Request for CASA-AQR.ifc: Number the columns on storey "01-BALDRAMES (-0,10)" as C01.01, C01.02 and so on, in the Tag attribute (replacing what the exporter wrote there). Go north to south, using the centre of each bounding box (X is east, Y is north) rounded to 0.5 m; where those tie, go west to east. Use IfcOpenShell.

First a look at what the model holds.

```python
import ifcopenshell
import ifcopenshell.util.element
import ifcopenshell.util.placement

model = ifcopenshell.open("CASA-AQR.ifc")
print(model.schema)
storey = next(s for s in model.by_type("IfcBuildingStorey") if s.Name == "01-BALDRAMES (-0,10)")
columns = [e for e in ifcopenshell.util.element.get_decomposition(storey) if e.is_a("IfcColumn")]
for e in sorted(columns, key=lambda e: e.id()):
    origin = ifcopenshell.util.placement.get_local_placement(e.ObjectPlacement)[:3, 3]
    print(e.id(), e.Tag, e.Name, origin.round(2) + 0.0, sep=" | ")
```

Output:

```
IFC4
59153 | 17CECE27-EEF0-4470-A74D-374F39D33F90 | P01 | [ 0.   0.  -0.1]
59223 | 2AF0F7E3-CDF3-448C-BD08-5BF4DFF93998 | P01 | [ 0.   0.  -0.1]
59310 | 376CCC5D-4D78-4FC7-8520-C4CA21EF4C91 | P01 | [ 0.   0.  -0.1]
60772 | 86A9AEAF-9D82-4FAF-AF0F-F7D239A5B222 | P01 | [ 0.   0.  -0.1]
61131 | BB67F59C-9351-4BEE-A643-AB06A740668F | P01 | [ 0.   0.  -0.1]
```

```python
import ifcopenshell
import ifcopenshell.geom
import ifcopenshell.util.element
import ifcopenshell.util.shape

model = ifcopenshell.open("CASA-AQR.ifc")
settings = ifcopenshell.geom.settings()
settings.set("use-world-coords", True)


def centre(element):
    shape = ifcopenshell.geom.create_shape(settings, element)
    return ifcopenshell.util.shape.get_bbox_centroid(shape.geometry)


storey = next(s for s in model.by_type("IfcBuildingStorey") if s.Name == "01-BALDRAMES (-0,10)")
columns = [e for e in ifcopenshell.util.element.get_decomposition(storey) if e.is_a("IfcColumn")]

# Insertion points can sit at a corner or the storey origin, so sort by the geometry (in metres).
centres = {e: centre(e) for e in columns}
columns.sort(key=lambda e: (-round(centres[e][1] / 0.5), centres[e][0]))

for i, e in enumerate(columns, start=1):
    number = f"C01.{i:02d}"
    e.Tag = number
    print(e.id(), number)

model.write("CASA-AQR-out.ifc")
```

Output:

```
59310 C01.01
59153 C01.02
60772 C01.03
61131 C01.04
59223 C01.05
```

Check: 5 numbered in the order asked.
